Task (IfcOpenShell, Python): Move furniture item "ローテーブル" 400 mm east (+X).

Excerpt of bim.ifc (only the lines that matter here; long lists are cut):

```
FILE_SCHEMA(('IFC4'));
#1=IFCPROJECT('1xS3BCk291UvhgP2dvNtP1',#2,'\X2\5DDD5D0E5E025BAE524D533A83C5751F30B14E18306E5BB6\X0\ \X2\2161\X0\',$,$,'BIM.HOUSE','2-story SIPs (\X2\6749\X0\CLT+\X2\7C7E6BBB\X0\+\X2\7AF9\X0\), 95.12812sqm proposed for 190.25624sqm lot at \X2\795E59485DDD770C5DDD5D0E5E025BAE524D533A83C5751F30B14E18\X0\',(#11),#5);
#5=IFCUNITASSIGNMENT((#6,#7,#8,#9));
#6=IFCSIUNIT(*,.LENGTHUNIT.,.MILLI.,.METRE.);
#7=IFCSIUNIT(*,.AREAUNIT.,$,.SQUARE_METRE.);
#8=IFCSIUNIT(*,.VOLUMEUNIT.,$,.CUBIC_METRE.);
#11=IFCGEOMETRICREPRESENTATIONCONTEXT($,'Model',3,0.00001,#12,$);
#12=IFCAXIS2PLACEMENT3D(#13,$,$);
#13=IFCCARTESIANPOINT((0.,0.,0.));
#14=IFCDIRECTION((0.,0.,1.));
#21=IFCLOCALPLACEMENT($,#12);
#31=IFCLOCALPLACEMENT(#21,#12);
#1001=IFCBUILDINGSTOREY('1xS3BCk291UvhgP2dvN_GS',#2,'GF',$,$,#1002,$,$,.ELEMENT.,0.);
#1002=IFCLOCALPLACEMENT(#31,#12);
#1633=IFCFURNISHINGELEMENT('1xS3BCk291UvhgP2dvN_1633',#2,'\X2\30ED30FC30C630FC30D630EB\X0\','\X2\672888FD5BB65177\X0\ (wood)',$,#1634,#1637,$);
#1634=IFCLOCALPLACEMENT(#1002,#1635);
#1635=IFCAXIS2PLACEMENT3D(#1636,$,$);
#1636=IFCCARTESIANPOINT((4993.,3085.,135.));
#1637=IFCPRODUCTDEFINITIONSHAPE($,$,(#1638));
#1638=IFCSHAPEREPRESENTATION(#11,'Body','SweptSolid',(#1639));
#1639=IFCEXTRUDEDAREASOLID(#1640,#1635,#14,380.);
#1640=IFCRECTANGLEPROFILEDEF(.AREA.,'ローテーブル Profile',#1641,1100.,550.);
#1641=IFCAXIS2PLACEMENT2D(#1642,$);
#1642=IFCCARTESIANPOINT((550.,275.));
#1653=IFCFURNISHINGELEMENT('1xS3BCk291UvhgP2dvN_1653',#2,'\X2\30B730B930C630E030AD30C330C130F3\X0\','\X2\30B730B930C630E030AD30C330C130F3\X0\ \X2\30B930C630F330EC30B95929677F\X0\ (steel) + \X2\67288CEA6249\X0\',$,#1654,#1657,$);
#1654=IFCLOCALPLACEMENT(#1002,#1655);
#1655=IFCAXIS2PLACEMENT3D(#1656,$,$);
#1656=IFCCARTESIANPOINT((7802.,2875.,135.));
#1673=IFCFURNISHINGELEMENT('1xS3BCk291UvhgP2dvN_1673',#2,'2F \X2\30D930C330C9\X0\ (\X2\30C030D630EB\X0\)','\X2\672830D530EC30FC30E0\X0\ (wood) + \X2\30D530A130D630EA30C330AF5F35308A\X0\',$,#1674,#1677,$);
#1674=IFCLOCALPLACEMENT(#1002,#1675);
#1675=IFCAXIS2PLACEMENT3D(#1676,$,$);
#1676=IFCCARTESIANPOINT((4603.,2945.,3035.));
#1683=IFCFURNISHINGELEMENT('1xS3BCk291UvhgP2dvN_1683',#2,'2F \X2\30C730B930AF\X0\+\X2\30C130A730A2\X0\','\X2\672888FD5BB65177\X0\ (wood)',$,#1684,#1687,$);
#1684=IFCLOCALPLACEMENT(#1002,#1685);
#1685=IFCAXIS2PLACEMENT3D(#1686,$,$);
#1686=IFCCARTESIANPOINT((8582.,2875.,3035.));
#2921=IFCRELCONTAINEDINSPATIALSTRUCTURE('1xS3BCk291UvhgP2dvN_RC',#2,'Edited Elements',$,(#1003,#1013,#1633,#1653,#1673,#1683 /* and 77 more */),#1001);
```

```python
import ifcopenshell
import ifcopenshell.api.geometry
import ifcopenshell.util.placement
import ifcopenshell.util.unit

model = ifcopenshell.open("bim.ifc")
unit_scale = ifcopenshell.util.unit.calculate_unit_scale(model)

item = model.by_guid("1xS3BCk291UvhgP2dvN_1633")
matrix = ifcopenshell.util.placement.get_local_placement(item.ObjectPlacement)
matrix[0, 3] += 0.4 / unit_scale
ifcopenshell.api.geometry.edit_object_placement(model, product=item, matrix=matrix, is_si=False)

print(ifcopenshell.util.placement.get_local_placement(item.ObjectPlacement).round(3) + 0.0)

model.write("bim_v2.ifc")
```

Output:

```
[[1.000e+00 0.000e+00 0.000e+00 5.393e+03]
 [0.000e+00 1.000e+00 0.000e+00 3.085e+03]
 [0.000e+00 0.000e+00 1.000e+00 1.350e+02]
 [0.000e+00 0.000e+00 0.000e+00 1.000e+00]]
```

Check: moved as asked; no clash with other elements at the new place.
